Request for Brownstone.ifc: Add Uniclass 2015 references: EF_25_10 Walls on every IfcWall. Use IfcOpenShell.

First a look at what the model holds.

```python
import ifcopenshell

model = ifcopenshell.open("Brownstone.ifc")
print(model.schema)
print("classifications:", [c.Name for c in model.by_type("IfcClassification")])
for ifc_class in ("IfcDoor", "IfcRoof", "IfcStair", "IfcWall", "IfcWindow"):
    print(ifc_class, len(model.by_type(ifc_class)))
```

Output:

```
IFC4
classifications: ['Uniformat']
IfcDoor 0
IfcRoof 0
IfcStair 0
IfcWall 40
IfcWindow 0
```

```python
import ifcopenshell
import ifcopenshell.api.classification

model = ifcopenshell.open("Brownstone.ifc")

system = ifcopenshell.api.classification.add_classification(model, classification="Uniclass 2015")

codes = {
    "IfcWall": ("EF_25_10", "Walls"),
}
for ifc_class, (code, name) in codes.items():
    products = model.by_type(ifc_class)
    ifcopenshell.api.classification.add_reference(
        model, products=products, classification=system, identification=code, name=name
    )
    print(code, len(products))

model.write("Brownstone_rev.ifc")
```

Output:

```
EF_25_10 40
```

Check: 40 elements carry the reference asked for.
